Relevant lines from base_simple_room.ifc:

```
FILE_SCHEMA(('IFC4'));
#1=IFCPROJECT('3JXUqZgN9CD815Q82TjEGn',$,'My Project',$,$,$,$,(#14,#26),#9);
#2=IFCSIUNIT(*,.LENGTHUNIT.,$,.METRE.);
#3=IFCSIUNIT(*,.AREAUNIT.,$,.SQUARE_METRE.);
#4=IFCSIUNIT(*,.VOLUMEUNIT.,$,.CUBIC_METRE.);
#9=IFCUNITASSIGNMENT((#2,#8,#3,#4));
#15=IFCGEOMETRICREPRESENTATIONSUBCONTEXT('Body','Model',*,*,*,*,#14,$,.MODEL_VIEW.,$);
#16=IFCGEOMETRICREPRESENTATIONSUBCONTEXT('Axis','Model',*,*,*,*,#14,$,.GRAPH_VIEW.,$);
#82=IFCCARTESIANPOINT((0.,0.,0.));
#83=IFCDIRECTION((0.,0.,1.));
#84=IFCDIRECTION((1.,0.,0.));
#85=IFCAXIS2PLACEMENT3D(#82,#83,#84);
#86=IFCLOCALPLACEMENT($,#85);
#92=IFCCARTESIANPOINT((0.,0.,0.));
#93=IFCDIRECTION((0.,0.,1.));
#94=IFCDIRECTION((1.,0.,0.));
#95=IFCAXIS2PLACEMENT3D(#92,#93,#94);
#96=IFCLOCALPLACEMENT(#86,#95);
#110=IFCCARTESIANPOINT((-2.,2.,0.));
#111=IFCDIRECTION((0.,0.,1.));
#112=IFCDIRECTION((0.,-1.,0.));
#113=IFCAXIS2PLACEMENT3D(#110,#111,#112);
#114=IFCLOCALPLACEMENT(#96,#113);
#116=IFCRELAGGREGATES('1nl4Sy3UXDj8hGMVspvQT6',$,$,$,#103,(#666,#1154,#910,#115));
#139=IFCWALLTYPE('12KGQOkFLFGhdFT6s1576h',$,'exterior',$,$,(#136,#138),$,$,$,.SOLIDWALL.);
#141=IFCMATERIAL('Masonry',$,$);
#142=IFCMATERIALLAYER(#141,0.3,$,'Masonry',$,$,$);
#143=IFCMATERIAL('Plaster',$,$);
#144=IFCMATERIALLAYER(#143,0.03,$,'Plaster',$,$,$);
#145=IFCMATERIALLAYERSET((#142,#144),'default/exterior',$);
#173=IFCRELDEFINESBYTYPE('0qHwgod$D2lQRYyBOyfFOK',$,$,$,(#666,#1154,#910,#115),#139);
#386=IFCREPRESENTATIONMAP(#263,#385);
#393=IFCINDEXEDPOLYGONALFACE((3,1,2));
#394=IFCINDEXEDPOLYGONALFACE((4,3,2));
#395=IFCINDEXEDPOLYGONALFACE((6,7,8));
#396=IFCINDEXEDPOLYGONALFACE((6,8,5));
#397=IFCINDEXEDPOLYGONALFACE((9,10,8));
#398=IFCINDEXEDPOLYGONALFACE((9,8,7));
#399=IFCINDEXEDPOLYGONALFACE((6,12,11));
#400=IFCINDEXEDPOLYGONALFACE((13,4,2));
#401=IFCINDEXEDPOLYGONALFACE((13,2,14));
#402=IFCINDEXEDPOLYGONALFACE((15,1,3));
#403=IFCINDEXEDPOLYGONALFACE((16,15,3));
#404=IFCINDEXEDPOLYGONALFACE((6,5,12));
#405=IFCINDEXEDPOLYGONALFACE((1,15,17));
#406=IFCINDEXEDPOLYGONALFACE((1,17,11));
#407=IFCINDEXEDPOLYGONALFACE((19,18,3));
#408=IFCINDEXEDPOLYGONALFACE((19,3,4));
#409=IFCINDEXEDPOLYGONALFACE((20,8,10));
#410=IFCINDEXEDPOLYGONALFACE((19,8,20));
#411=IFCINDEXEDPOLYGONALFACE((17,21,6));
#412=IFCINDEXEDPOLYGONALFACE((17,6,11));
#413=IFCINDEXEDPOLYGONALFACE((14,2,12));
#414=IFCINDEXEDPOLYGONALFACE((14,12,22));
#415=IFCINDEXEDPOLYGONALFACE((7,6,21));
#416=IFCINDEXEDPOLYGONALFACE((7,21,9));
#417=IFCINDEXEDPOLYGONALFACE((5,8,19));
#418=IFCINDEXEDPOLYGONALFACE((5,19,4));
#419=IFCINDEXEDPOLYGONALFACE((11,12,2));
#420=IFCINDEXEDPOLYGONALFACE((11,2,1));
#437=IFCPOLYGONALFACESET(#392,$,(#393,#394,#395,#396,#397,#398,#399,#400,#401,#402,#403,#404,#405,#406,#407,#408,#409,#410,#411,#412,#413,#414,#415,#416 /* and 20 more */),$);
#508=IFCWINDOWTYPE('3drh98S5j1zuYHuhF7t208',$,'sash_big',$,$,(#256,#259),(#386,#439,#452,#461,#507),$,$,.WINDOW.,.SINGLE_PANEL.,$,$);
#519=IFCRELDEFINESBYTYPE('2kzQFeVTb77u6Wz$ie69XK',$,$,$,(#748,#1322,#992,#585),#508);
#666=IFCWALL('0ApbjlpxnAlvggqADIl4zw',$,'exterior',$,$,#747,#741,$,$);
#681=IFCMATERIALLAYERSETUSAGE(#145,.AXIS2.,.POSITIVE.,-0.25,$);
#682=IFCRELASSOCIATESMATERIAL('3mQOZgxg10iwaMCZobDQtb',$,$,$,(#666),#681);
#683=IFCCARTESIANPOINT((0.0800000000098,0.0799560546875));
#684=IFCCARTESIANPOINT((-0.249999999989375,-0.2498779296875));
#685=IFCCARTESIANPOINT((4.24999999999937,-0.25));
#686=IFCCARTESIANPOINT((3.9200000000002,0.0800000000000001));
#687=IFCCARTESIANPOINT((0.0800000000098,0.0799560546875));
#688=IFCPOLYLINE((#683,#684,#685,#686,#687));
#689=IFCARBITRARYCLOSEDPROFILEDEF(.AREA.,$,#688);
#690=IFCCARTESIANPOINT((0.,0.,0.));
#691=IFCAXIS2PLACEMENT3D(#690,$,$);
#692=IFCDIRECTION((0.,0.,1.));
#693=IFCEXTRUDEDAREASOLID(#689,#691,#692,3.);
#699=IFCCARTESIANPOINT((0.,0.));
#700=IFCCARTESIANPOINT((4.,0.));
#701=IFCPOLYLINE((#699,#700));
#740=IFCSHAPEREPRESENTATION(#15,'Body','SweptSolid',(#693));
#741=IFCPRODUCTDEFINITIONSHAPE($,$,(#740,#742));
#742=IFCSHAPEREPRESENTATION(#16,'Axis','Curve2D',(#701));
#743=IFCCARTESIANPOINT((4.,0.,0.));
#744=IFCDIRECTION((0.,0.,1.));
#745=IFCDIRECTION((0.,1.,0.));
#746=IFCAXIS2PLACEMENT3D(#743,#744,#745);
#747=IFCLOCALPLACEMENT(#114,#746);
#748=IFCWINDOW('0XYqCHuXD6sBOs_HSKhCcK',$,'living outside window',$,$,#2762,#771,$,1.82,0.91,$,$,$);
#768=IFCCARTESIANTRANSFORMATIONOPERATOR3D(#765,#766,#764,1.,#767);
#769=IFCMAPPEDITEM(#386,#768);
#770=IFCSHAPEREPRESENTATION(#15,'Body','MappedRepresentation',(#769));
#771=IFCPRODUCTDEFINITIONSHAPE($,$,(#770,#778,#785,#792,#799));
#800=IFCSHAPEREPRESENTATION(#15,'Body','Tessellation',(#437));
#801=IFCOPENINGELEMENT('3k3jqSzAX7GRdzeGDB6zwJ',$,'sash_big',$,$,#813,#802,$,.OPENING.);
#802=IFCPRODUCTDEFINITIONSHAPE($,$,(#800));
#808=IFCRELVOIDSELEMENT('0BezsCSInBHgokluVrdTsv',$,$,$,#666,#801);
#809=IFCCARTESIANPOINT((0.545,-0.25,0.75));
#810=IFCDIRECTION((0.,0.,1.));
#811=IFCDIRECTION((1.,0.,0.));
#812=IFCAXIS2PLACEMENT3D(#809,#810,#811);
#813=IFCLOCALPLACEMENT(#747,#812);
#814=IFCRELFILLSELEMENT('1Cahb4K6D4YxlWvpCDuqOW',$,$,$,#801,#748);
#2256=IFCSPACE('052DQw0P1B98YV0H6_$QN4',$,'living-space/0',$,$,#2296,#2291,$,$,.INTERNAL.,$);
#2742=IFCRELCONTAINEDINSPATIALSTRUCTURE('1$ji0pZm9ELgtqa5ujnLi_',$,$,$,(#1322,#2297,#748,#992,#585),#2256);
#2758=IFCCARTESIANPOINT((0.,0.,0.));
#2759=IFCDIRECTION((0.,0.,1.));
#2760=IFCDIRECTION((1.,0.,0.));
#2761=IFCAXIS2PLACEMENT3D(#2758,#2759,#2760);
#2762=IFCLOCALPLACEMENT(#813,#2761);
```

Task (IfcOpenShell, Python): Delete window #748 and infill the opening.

```python
import ifcopenshell
import ifcopenshell.api.feature
import ifcopenshell.api.root
import ifcopenshell.geom
import ifcopenshell.util.shape

model = ifcopenshell.open("base_simple_room.ifc")
settings = ifcopenshell.geom.settings()


def volume(element):
    """Net volume in cubic metres, openings subtracted."""
    shape = ifcopenshell.geom.create_shape(settings, element)
    return ifcopenshell.util.shape.get_volume(shape.geometry)


window = model.by_guid("0XYqCHuXD6sBOs_HSKhCcK")
opening = window.FillsVoids[0].RelatingOpeningElement
wall = opening.VoidsElements[0].RelatingBuildingElement
before = volume(wall)

ifcopenshell.api.root.remove_product(model, product=window)
ifcopenshell.api.feature.remove_feature(model, feature=opening)

after = volume(wall)

print(f"wall volume {before:.3f} -> {after:.3f} m3")

model.write("base_simple_room_edited.ifc")
```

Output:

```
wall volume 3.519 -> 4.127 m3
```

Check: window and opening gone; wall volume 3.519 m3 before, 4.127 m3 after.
